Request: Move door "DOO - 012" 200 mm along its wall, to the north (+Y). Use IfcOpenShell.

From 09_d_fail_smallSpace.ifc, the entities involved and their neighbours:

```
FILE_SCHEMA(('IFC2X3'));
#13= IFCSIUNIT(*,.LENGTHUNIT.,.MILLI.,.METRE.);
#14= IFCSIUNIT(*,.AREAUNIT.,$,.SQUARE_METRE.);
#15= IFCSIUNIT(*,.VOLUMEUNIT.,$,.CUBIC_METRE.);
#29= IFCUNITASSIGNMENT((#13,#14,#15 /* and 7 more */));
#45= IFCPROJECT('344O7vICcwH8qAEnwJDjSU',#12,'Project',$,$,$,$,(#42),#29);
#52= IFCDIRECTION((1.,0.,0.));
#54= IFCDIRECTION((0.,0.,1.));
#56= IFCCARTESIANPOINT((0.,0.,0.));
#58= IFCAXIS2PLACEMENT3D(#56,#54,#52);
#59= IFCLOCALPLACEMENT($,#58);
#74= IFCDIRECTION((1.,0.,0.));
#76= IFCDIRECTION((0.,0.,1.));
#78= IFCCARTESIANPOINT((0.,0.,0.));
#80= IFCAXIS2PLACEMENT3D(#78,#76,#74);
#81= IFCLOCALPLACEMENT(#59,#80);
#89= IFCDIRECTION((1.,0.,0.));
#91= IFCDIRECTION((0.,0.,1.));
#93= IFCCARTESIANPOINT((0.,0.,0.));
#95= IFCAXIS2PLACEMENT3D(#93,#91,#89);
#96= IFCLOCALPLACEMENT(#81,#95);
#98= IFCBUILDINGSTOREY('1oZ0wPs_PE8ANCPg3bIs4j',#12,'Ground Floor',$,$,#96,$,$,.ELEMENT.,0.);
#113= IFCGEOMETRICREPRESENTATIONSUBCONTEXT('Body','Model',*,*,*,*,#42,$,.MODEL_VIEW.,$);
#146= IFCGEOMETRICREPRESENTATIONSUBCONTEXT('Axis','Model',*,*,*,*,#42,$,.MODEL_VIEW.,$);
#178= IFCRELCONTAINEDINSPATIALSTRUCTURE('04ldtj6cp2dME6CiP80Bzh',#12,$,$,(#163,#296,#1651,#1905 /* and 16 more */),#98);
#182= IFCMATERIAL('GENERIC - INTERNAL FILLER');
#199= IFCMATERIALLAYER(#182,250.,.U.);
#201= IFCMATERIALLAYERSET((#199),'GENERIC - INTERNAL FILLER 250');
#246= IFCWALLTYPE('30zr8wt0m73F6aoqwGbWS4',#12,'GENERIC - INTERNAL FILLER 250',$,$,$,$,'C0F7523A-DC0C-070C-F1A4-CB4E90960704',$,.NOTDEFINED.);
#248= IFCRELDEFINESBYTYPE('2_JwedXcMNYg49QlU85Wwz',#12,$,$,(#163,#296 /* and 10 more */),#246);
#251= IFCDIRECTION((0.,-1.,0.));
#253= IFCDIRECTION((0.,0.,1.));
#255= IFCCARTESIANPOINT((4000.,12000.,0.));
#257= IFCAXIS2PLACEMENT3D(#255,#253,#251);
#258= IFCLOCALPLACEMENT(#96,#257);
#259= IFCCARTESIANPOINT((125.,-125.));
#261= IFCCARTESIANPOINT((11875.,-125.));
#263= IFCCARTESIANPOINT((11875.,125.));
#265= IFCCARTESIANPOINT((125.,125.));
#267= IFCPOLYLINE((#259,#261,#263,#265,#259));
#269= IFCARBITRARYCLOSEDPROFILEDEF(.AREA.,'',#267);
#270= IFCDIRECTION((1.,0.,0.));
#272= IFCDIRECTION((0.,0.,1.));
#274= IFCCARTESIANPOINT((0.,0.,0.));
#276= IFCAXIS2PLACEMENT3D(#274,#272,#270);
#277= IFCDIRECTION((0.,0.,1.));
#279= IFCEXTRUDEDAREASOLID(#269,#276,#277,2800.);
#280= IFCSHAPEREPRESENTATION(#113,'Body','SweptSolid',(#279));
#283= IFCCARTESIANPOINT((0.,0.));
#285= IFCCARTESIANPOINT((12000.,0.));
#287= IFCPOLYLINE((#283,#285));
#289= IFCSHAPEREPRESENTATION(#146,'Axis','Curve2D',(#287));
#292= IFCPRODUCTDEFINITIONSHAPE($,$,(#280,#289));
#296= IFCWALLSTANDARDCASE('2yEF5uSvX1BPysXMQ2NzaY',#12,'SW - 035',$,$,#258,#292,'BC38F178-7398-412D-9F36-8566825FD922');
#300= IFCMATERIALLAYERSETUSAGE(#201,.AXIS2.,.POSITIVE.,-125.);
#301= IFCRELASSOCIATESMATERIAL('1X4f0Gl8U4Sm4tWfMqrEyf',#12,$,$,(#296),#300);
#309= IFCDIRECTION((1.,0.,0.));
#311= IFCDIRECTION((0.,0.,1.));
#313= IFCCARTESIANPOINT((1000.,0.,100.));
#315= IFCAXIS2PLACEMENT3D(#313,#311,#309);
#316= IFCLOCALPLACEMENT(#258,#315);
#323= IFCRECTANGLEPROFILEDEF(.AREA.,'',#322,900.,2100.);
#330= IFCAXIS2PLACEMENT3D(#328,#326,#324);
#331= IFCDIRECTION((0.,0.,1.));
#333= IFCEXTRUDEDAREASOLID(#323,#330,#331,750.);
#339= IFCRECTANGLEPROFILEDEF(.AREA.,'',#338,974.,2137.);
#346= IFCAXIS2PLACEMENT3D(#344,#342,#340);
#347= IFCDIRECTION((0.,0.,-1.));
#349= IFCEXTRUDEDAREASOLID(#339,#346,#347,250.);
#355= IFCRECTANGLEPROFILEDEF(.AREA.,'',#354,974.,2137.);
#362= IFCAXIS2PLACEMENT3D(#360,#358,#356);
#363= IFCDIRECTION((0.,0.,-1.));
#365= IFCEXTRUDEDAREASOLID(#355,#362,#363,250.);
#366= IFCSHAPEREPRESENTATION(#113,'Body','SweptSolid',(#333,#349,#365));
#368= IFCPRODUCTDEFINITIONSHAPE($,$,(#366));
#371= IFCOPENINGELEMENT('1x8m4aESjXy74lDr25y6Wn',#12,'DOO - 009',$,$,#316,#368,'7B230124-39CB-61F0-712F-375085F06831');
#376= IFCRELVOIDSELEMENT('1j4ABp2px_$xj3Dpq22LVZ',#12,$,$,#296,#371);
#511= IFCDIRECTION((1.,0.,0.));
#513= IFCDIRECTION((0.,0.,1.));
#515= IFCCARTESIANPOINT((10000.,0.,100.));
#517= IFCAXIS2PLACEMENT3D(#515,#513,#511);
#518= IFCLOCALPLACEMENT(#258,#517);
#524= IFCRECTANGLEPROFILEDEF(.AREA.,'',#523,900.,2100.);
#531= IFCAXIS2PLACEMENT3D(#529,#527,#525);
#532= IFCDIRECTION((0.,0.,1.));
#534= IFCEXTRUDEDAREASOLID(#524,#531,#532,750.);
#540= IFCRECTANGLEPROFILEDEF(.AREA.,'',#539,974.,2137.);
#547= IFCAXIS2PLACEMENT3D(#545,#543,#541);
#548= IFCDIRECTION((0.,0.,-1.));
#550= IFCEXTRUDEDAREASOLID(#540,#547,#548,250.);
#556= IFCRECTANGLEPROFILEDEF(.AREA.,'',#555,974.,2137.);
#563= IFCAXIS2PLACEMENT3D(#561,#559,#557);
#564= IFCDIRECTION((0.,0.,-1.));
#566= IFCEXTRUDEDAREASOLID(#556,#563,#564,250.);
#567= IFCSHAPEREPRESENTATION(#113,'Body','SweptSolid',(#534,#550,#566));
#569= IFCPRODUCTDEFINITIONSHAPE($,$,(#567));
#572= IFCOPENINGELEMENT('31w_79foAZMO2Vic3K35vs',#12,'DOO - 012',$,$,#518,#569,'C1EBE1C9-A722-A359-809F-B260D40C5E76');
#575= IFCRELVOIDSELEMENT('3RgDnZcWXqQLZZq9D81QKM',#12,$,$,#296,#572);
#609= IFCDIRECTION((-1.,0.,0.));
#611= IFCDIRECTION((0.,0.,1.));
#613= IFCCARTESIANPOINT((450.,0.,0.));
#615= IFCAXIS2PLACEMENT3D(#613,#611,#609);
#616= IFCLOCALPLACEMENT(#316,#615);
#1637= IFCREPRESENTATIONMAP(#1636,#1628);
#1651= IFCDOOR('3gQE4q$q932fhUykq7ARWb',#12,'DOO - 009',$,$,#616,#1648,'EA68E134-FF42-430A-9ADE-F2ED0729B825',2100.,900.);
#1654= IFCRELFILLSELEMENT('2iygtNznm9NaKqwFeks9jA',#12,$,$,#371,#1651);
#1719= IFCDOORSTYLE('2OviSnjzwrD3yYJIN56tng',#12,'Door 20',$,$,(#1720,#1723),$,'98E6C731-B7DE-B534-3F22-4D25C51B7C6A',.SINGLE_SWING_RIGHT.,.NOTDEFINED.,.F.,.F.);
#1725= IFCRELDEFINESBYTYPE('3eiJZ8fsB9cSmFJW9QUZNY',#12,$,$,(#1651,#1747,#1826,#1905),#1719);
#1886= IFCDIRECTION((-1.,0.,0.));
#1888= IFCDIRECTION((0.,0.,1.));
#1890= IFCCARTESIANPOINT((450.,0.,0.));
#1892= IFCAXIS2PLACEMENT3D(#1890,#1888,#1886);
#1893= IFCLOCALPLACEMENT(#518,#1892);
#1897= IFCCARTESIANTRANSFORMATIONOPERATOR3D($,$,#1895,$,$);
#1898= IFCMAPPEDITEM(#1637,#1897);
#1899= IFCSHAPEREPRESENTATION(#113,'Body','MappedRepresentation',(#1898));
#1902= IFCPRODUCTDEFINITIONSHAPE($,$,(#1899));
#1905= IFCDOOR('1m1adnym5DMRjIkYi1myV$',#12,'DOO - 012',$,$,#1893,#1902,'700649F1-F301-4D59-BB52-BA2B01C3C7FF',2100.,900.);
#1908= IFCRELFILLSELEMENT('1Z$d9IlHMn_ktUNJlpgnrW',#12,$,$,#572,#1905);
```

```python
import ifcopenshell
import ifcopenshell.api.geometry
import ifcopenshell.util.placement

model = ifcopenshell.open("09_d_fail_smallSpace.ifc")

door = model.by_guid("1m1adnym5DMRjIkYi1myV$")
opening = door.FillsVoids[0].RelatingOpeningElement
wall = opening.VoidsElements[0].RelatingBuildingElement

wall_matrix = ifcopenshell.util.placement.get_local_placement(wall.ObjectPlacement)
shift = wall_matrix[:3, 0] * -200.0
before = ifcopenshell.util.placement.get_local_placement(door.ObjectPlacement)[:3, 3].copy()

# The door is placed relative to its opening, so it follows when the opening moves.
matrix = ifcopenshell.util.placement.get_local_placement(opening.ObjectPlacement)
matrix[:3, 3] += shift
ifcopenshell.api.geometry.edit_object_placement(
    model, product=opening, matrix=matrix, is_si=False, should_transform_children=True
)

after = ifcopenshell.util.placement.get_local_placement(door.ObjectPlacement)[:3, 3]
print("door moved by", (after - before).round(3) + 0.0)

model.write("09_d_fail_smallSpace_updated.ifc")
```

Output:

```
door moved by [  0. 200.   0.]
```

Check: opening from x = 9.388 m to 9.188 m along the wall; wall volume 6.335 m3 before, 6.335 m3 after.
